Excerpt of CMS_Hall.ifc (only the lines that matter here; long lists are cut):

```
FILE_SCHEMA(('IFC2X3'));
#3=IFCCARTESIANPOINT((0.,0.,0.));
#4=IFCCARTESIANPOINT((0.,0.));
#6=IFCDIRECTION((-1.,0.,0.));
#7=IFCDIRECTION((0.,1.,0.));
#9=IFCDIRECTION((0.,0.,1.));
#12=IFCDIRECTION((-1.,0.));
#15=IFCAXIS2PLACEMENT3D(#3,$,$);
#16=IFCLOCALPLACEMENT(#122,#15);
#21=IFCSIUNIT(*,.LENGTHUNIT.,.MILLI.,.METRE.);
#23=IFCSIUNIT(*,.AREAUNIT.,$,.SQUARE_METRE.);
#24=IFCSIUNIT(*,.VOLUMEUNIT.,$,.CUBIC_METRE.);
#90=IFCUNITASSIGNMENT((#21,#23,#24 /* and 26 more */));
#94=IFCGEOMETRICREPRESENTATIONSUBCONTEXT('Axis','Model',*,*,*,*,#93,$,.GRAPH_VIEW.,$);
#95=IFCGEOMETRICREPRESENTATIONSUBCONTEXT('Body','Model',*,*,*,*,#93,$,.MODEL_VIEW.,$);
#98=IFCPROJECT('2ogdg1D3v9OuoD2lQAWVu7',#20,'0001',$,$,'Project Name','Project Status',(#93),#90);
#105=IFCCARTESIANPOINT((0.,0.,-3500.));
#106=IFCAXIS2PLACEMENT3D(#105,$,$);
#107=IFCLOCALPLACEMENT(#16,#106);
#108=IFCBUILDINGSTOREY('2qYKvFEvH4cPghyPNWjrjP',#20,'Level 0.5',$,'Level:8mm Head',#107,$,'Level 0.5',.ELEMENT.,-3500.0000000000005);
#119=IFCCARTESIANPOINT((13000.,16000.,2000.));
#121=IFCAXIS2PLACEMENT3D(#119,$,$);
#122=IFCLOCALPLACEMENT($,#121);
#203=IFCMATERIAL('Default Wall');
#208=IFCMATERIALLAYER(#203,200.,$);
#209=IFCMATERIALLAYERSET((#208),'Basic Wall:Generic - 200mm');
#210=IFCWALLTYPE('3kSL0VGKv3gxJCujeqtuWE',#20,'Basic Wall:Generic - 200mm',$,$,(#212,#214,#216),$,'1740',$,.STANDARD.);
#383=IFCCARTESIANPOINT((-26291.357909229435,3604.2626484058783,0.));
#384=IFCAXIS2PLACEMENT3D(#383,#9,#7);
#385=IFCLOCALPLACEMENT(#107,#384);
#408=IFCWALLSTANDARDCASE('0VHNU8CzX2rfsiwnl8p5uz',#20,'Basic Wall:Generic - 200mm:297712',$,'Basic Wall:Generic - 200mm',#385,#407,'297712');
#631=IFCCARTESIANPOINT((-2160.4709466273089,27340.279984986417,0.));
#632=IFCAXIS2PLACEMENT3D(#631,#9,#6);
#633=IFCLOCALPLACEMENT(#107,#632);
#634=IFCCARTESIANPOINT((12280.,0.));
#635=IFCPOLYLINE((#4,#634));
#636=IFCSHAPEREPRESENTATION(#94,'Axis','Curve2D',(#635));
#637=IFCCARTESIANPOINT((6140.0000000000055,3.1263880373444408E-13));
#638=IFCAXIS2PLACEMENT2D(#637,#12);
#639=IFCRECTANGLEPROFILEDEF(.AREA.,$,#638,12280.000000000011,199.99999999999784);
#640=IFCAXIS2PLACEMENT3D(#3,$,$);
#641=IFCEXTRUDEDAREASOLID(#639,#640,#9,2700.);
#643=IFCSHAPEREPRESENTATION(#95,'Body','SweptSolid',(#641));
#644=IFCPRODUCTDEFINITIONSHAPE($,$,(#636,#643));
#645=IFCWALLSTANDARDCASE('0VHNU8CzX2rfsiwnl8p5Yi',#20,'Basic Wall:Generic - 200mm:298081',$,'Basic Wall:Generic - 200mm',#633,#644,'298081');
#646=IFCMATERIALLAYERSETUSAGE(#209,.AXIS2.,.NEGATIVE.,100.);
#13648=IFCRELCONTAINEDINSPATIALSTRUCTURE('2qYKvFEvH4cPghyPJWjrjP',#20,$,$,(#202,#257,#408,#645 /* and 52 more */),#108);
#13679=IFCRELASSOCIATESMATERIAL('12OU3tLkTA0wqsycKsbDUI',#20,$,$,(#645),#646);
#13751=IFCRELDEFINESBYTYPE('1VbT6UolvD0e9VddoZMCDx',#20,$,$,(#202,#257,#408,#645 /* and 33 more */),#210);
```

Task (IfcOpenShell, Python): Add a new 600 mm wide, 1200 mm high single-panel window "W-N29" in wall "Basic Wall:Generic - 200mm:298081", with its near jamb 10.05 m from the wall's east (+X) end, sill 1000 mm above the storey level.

```python
import numpy as np
import ifcopenshell
import ifcopenshell.api.feature
import ifcopenshell.api.geometry
import ifcopenshell.api.root
import ifcopenshell.api.spatial
import ifcopenshell.api.type
import ifcopenshell.geom
import ifcopenshell.util.element
import ifcopenshell.util.placement
import ifcopenshell.util.representation
import ifcopenshell.util.shape
import ifcopenshell.util.unit

model = ifcopenshell.open("CMS_Hall.ifc")
unit_scale = ifcopenshell.util.unit.calculate_unit_scale(model)
settings = ifcopenshell.geom.settings()


def volume(element):
    """Net volume in cubic metres, openings subtracted."""
    shape = ifcopenshell.geom.create_shape(settings, element)
    return ifcopenshell.util.shape.get_volume(shape.geometry)


wall = model.by_guid("0VHNU8CzX2rfsiwnl8p5Yi")
storey = ifcopenshell.util.element.get_container(wall, ifc_class="IfcBuildingStorey")
context = ifcopenshell.util.representation.get_context(model, "Model", "Body", "MODEL_VIEW")
before = volume(wall)

width, height, from_end, sill = 0.6, 1.2, 10.05, 1  # metres

# The wall runs along its own X axis, and the end named is its -X end.
wall_shape = ifcopenshell.geom.create_shape(settings, wall)
x, y, z = ifcopenshell.util.shape.get_vertices(wall_shape.geometry).T
start = x.min() + from_end
face, thickness = float(y.min()), float(y.max() - y.min())
wall_matrix = ifcopenshell.util.placement.get_local_placement(wall.ObjectPlacement)
level = ifcopenshell.util.placement.get_local_placement(storey.ObjectPlacement)[2, 3]


def in_wall(x, y):
    """Placement at x, y metres in the wall's axes, at sill height."""
    matrix = wall_matrix.copy()
    matrix[:, 3] = wall_matrix @ np.array([x / unit_scale, y / unit_scale, 0.0, 1.0])
    matrix[2, 3] = level + sill / unit_scale
    return matrix


# Opening: a box that overshoots both wall faces by 50 mm.
opening = ifcopenshell.api.root.create_entity(model, ifc_class="IfcOpeningElement")
box = ifcopenshell.api.geometry.add_wall_representation(
    model, context=context, length=width, height=height, thickness=thickness + 0.1
)
ifcopenshell.api.geometry.assign_representation(model, product=opening, representation=box)
ifcopenshell.api.geometry.edit_object_placement(model, product=opening, matrix=in_wall(start, face - 0.05), is_si=False)
ifcopenshell.api.feature.add_feature(model, feature=opening, element=wall)

window = ifcopenshell.api.root.create_entity(model, ifc_class="IfcWindow", name="W-N29")
window.OverallWidth, window.OverallHeight = width / unit_scale, height / unit_scale
body = ifcopenshell.api.geometry.add_window_representation(
    model,
    context=context,
    overall_width=window.OverallWidth,
    overall_height=window.OverallHeight,
    partition_type="SINGLE_PANEL",
)
ifcopenshell.api.geometry.assign_representation(model, product=window, representation=body)
ifcopenshell.api.spatial.assign_container(model, products=[window], relating_structure=storey)
fills = ifcopenshell.api.feature.add_filling(model, opening=opening, element=window)
fills.OwnerHistory = window.OwnerHistory  # required in IFC2X3

# IFC2X3 keeps the operation on the window style.
style = ifcopenshell.api.root.create_entity(model, ifc_class="IfcWindowStyle", name="W-N29")
style.OperationType, style.ConstructionType = "SINGLE_PANEL", "NOTDEFINED"
style.ParameterTakesPrecedence = style.Sizeable = False
ifcopenshell.api.type.assign_type(model, related_objects=[window], relating_type=style)

# Centre the window in the wall's thickness.
ifcopenshell.api.geometry.edit_object_placement(model, product=window, matrix=in_wall(start, face), is_si=False)
window_shape = ifcopenshell.geom.create_shape(settings, window)
depth = ifcopenshell.util.shape.get_vertices(window_shape.geometry)[:, 1]
offset = face + thickness / 2 - (depth.min() + depth.max()) / 2
ifcopenshell.api.geometry.edit_object_placement(model, product=window, matrix=in_wall(start, offset), is_si=False)

after = volume(wall)

print(f"wall volume {before:.3f} -> {after:.3f} m3")

model.write("CMS_Hall_updated.ifc")
```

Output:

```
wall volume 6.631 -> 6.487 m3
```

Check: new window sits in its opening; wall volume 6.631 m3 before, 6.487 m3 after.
